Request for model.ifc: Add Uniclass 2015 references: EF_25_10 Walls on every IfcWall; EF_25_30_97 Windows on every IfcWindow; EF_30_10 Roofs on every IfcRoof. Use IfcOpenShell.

First a look at what the model holds.

```python
import ifcopenshell

model = ifcopenshell.open("model.ifc")
print(model.schema)
print("classifications:", [c.Name for c in model.by_type("IfcClassification")])
for ifc_class in ("IfcDoor", "IfcRoof", "IfcStair", "IfcWall", "IfcWindow"):
    print(ifc_class, len(model.by_type(ifc_class)))
```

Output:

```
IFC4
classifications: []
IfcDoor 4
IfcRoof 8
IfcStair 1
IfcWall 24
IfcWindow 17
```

```python
import ifcopenshell
import ifcopenshell.api.classification

model = ifcopenshell.open("model.ifc")

system = ifcopenshell.api.classification.add_classification(model, classification="Uniclass 2015")

codes = {
    "IfcWall": ("EF_25_10", "Walls"),
    "IfcWindow": ("EF_25_30_97", "Windows"),
    "IfcRoof": ("EF_30_10", "Roofs"),
}
for ifc_class, (code, name) in codes.items():
    products = model.by_type(ifc_class)
    ifcopenshell.api.classification.add_reference(
        model, products=products, classification=system, identification=code, name=name
    )
    print(code, len(products))

model.write("model-out.ifc")
```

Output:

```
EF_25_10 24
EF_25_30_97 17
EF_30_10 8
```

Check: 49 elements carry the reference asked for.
